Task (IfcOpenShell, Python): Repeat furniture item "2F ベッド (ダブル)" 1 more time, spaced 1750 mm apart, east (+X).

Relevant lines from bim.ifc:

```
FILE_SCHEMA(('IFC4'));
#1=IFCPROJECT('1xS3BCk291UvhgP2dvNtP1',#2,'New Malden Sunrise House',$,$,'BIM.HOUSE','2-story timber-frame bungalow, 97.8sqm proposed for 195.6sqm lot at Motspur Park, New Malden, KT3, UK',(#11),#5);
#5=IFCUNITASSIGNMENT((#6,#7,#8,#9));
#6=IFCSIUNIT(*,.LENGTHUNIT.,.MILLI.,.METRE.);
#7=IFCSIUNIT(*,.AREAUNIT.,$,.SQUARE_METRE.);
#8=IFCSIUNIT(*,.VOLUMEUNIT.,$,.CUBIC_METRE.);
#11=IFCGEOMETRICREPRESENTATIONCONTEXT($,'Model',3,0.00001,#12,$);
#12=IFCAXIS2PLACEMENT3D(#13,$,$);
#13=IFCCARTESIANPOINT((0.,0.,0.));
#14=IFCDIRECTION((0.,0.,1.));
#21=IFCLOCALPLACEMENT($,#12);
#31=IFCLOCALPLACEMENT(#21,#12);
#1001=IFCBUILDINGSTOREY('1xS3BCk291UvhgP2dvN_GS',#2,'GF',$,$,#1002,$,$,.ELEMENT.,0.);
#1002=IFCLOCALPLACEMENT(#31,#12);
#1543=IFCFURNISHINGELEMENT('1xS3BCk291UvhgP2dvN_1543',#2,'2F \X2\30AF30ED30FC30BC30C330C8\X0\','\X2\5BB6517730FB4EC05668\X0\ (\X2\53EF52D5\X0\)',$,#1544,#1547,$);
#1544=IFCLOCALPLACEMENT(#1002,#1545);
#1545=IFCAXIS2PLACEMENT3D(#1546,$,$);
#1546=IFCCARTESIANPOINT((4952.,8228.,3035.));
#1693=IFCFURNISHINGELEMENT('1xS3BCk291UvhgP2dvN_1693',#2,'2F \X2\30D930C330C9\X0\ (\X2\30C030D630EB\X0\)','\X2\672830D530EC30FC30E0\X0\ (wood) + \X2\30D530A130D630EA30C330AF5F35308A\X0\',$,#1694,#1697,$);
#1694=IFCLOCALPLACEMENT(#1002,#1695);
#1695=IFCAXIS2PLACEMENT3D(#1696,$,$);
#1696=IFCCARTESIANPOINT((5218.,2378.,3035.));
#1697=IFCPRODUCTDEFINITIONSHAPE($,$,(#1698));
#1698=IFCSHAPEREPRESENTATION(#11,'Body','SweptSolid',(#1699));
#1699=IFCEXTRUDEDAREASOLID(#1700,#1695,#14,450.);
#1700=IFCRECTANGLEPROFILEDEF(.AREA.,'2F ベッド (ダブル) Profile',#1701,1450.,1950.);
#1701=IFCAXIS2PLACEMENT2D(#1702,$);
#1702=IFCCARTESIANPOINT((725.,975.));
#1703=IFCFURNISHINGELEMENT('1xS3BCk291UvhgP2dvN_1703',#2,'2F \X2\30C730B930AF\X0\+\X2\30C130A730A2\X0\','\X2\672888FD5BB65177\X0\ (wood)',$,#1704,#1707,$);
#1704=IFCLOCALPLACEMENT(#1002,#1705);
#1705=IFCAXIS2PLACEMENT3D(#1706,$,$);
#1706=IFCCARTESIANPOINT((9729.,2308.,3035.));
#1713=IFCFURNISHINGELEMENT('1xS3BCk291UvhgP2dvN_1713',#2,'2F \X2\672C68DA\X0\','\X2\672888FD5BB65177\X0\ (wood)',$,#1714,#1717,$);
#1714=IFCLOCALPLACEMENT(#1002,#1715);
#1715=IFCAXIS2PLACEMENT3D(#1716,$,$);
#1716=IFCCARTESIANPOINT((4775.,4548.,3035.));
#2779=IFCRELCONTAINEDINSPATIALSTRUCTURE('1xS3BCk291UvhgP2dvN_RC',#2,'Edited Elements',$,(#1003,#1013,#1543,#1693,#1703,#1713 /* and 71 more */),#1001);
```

```python
import numpy as np
import ifcopenshell
import ifcopenshell.api.geometry
import ifcopenshell.api.root
import ifcopenshell.util.element
import ifcopenshell.util.placement
import ifcopenshell.util.unit

model = ifcopenshell.open("bim.ifc")
unit_scale = ifcopenshell.util.unit.calculate_unit_scale(model)


def reuse_history(source, copy):
    """copy_class also copies each property set's owner history, people and application; keep the originals."""
    for rel in copy.IsDefinedBy:
        if rel.is_a("IfcRelDefinesByProperties") and (history := rel.RelatingPropertyDefinition.OwnerHistory):
            rel.RelatingPropertyDefinition.OwnerHistory = source.OwnerHistory
            ifcopenshell.util.element.remove_deep2(model, history)


source = model.by_guid("1xS3BCk291UvhgP2dvN_1693")
base = ifcopenshell.util.placement.get_local_placement(source.ObjectPlacement)
step = np.array([1.0, 0.0, 0.0]) * 1.75 / unit_scale

for i in range(1, 2):
    copy = ifcopenshell.api.root.copy_class(model, product=source)
    copy.Representation = ifcopenshell.util.element.copy_deep(
        model, source.Representation, exclude=["IfcGeometricRepresentationContext", "IfcRepresentationMap"]
    )
    reuse_history(source, copy)
    matrix = base.copy()
    matrix[:3, 3] += i * step
    print("added at", matrix[:3, 3].round(3) + 0.0)
    ifcopenshell.api.geometry.edit_object_placement(model, product=copy, matrix=matrix, is_si=False)

model.write("bim_v2.ifc")
```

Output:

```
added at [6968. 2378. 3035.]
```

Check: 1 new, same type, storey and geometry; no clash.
